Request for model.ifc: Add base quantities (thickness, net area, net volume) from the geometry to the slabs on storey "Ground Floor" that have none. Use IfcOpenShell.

First a look at what the model holds.

```python
import ifcopenshell
import ifcopenshell.util.element
import ifcopenshell.util.unit

model = ifcopenshell.open("model.ifc")
print(model.schema)
for unit_type in ("LENGTHUNIT", "AREAUNIT", "VOLUMEUNIT"):
    print(unit_type, ifcopenshell.util.unit.calculate_unit_scale(model, unit_type))
storey = next(s for s in model.by_type("IfcBuildingStorey") if s.Name == "Ground Floor")
slabs = [e for e in ifcopenshell.util.element.get_decomposition(storey) if e.is_a("IfcSlab")]
for e in sorted(slabs, key=lambda e: e.id()):
    print(e.id(), e.is_a(), e.Name, list(ifcopenshell.util.element.get_psets(e, qtos_only=True)), sep=" | ")
```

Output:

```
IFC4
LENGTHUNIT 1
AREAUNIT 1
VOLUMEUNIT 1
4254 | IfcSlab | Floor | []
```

```python
import ifcopenshell
import ifcopenshell.api.pset
import ifcopenshell.geom
import ifcopenshell.util.element
import ifcopenshell.util.shape
import ifcopenshell.util.unit

model = ifcopenshell.open("model.ifc")
unit_scale = ifcopenshell.util.unit.calculate_unit_scale(model)
area_scale = ifcopenshell.util.unit.calculate_unit_scale(model, "AREAUNIT")
volume_scale = ifcopenshell.util.unit.calculate_unit_scale(model, "VOLUMEUNIT")
settings = ifcopenshell.geom.settings()

storey = next(s for s in model.by_type("IfcBuildingStorey") if s.Name == "Ground Floor")
slabs = [e for e in ifcopenshell.util.element.get_decomposition(storey) if e.is_a("IfcSlab")]

for e in sorted(slabs, key=lambda e: e.id()):
    if ifcopenshell.util.element.get_psets(e, qtos_only=True, should_inherit=False):
        continue
    # Geometry comes back in metres, in the element's own axes.
    shape = ifcopenshell.geom.create_shape(settings, e)
    values = {
        "Width": ifcopenshell.util.shape.get_z(shape.geometry) / unit_scale,
        "NetArea": ifcopenshell.util.shape.get_footprint_area(shape.geometry) / area_scale,
        "NetVolume": ifcopenshell.util.shape.get_volume(shape.geometry) / volume_scale,
    }
    qto = ifcopenshell.api.pset.add_qto(model, product=e, name="Qto_SlabBaseQuantities")
    ifcopenshell.api.pset.edit_qto(model, qto=qto, properties=values)
    print(e.id(), {k: round(v, 3) for k, v in values.items()})

model.write("model_rev.ifc")
```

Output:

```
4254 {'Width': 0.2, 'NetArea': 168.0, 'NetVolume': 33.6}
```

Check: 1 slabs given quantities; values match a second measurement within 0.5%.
